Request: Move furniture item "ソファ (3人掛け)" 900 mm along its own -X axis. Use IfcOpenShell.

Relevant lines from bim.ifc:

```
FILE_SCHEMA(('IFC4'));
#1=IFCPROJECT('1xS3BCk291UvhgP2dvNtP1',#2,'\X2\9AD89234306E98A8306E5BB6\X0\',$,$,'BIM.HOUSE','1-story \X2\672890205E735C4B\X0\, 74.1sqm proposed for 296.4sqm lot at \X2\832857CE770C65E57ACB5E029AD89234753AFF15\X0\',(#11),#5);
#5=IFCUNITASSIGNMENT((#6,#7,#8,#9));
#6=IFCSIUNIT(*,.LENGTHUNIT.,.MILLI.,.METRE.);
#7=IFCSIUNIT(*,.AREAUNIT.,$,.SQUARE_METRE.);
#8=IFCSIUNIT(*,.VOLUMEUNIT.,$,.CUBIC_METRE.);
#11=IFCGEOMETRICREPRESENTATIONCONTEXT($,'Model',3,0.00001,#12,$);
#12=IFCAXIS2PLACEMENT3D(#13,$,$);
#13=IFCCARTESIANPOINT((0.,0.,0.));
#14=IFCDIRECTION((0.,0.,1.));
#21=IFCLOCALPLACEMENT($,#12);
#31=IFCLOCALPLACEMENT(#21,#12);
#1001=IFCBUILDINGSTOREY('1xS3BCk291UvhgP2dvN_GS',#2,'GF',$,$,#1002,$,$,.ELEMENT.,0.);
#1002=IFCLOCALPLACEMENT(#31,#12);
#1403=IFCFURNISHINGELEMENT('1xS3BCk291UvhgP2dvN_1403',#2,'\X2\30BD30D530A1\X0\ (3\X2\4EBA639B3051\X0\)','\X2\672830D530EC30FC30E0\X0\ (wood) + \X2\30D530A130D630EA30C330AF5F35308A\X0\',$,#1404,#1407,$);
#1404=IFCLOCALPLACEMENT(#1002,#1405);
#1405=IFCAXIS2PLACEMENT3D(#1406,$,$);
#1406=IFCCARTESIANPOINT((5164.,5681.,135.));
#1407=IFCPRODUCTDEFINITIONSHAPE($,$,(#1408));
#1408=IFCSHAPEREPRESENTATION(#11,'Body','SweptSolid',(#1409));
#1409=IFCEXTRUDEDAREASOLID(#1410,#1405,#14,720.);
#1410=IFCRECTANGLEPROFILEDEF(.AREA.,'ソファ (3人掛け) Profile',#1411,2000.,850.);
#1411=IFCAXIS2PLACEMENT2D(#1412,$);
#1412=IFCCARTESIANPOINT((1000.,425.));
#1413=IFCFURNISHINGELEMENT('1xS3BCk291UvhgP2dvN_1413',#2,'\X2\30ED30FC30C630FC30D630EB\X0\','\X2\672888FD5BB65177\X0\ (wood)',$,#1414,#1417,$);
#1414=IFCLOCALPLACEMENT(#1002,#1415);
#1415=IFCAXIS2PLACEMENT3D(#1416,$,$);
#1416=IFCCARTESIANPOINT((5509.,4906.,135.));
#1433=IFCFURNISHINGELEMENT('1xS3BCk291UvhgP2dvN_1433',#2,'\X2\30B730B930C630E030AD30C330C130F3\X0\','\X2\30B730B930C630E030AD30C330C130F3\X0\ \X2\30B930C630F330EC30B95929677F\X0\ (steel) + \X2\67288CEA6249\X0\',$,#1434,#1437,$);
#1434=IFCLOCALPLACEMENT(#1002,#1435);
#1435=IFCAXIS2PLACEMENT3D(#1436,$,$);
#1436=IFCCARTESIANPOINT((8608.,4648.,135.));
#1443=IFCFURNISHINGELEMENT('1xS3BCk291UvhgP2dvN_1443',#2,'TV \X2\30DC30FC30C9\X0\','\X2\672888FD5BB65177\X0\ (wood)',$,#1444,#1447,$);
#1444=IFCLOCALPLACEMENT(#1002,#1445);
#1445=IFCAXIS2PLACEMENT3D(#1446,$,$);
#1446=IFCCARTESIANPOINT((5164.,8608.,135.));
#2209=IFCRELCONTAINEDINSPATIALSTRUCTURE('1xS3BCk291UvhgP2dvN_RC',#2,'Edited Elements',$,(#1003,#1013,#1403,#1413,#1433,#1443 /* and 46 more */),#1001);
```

```python
import ifcopenshell
import ifcopenshell.api.geometry
import ifcopenshell.util.placement
import ifcopenshell.util.unit

model = ifcopenshell.open("bim.ifc")
unit_scale = ifcopenshell.util.unit.calculate_unit_scale(model)

item = model.by_guid("1xS3BCk291UvhgP2dvN_1403")
matrix = ifcopenshell.util.placement.get_local_placement(item.ObjectPlacement)
matrix[:3, 3] -= matrix[:3, 0] * 0.9 / unit_scale
ifcopenshell.api.geometry.edit_object_placement(model, product=item, matrix=matrix, is_si=False)

print(ifcopenshell.util.placement.get_local_placement(item.ObjectPlacement).round(3) + 0.0)

model.write("bim_rev.ifc")
```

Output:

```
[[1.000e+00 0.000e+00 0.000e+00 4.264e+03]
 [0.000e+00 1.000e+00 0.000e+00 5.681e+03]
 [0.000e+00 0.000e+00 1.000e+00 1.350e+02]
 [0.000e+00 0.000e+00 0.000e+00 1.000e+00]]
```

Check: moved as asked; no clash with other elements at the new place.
